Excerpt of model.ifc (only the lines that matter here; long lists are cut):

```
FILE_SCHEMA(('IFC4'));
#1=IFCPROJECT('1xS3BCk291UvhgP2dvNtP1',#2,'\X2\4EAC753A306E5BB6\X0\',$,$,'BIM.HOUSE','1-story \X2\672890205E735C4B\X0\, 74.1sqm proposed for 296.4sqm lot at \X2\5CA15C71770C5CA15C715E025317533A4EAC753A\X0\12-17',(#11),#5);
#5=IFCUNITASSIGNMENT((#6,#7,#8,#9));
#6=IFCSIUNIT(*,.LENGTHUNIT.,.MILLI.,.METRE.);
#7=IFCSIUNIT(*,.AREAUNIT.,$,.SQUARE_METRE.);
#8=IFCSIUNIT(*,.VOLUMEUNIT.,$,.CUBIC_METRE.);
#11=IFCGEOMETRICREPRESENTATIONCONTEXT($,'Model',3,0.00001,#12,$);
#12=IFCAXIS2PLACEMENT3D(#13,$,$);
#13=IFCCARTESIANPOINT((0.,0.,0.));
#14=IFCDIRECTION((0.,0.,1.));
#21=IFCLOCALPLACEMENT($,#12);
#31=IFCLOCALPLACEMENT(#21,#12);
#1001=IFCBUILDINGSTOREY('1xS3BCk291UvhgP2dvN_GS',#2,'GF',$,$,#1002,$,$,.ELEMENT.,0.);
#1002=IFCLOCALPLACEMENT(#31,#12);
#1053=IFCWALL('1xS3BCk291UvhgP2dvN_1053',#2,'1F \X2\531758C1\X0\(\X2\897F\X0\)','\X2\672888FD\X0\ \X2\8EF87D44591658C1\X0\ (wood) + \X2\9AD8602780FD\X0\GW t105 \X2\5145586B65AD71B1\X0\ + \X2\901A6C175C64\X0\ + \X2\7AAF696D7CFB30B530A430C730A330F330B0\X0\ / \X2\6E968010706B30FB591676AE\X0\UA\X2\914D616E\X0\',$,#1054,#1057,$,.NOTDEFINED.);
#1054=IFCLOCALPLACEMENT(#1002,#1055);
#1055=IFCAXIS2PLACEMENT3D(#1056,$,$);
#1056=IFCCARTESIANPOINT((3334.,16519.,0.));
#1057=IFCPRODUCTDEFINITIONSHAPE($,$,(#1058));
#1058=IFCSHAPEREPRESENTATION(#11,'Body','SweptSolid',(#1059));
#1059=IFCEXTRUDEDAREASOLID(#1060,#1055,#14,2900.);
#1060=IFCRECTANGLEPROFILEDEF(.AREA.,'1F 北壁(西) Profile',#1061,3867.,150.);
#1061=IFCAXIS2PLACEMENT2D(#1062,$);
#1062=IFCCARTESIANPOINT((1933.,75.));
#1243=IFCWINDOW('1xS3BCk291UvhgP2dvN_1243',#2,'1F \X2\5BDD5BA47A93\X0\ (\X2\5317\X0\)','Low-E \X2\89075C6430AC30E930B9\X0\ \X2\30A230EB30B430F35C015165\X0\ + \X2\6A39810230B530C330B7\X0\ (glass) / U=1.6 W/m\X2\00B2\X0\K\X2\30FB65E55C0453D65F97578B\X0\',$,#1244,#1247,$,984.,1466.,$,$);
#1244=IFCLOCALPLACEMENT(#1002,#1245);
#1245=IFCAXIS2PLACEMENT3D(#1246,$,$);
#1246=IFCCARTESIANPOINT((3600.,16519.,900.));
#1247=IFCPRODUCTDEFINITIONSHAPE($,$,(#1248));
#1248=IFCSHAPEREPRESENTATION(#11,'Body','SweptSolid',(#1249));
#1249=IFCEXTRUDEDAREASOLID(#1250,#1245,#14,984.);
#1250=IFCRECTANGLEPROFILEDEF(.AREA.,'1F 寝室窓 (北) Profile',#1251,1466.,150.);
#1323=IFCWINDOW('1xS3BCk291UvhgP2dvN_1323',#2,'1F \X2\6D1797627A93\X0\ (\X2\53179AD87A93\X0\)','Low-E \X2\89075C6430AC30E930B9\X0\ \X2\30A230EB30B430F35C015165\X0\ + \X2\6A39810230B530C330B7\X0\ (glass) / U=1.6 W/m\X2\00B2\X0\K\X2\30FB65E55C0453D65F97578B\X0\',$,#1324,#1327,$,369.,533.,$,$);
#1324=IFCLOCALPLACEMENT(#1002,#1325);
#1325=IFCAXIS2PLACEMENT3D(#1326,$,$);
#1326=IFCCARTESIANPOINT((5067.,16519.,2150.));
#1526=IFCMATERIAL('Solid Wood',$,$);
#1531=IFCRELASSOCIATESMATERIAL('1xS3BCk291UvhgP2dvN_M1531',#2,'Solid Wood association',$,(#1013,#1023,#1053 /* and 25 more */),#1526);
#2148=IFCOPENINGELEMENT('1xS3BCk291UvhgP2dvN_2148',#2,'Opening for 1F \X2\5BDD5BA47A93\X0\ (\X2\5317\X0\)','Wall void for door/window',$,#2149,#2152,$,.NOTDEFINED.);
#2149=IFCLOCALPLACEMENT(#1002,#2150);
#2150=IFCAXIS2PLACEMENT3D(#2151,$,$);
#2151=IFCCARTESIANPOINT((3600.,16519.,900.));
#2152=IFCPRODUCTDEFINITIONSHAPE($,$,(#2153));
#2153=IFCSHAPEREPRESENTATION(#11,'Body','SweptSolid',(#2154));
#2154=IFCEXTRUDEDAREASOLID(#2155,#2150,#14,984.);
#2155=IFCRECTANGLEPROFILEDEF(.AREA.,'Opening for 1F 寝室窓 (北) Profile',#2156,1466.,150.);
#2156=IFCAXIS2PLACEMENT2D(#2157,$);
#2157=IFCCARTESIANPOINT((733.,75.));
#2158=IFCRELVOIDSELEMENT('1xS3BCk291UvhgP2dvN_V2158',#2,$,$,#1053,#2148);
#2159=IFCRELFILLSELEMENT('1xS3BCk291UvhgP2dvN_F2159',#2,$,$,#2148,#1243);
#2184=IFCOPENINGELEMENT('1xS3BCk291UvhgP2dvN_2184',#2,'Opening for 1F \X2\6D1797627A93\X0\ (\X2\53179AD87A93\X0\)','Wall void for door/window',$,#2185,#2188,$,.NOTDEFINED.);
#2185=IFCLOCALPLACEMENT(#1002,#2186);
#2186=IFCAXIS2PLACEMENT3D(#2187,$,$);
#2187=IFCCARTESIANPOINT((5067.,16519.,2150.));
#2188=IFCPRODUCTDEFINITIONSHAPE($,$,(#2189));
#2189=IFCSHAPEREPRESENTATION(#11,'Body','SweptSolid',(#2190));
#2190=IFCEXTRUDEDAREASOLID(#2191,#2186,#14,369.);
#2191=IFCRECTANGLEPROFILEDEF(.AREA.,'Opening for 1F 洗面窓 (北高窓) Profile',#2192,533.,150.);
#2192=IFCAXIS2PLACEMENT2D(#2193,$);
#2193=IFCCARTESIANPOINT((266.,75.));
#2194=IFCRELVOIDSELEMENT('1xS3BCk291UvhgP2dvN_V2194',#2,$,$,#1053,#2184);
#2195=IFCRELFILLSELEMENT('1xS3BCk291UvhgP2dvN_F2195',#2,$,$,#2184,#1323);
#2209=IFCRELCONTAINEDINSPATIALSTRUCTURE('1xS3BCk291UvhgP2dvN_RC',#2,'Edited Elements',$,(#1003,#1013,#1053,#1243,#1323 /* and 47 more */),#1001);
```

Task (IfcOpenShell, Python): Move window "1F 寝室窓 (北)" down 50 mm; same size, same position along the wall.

```python
import numpy as np
import ifcopenshell
import ifcopenshell.api.geometry
import ifcopenshell.util.placement
import ifcopenshell.util.unit

model = ifcopenshell.open("model.ifc")
unit_scale = ifcopenshell.util.unit.calculate_unit_scale(model)

window = model.by_guid("1xS3BCk291UvhgP2dvN_1243")
opening = window.FillsVoids[0].RelatingOpeningElement
dz = -0.05 / unit_scale

shift = np.array([0.0, 0.0, dz])
# The window is not placed relative to its opening, so move both.
for product in (opening, window):
    matrix = ifcopenshell.util.placement.get_local_placement(product.ObjectPlacement)
    matrix[:3, 3] += shift
    ifcopenshell.api.geometry.edit_object_placement(model, product=product, matrix=matrix, is_si=False)

print(f"moved by {dz * unit_scale:+.3f} m")

model.write("model_edited.ifc")
```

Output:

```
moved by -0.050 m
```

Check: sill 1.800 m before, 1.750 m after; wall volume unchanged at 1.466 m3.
